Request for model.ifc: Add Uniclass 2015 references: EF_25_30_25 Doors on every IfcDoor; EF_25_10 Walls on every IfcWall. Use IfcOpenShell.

First a look at what the model holds.

```python
import ifcopenshell

model = ifcopenshell.open("model.ifc")
print(model.schema)
print("classifications:", [c.Name for c in model.by_type("IfcClassification")])
for ifc_class in ("IfcDoor", "IfcRoof", "IfcStair", "IfcWall", "IfcWindow"):
    print(ifc_class, len(model.by_type(ifc_class)))
```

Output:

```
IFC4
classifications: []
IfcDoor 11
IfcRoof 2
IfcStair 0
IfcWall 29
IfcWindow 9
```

```python
import ifcopenshell
import ifcopenshell.api.classification

model = ifcopenshell.open("model.ifc")

system = ifcopenshell.api.classification.add_classification(model, classification="Uniclass 2015")

codes = {
    "IfcDoor": ("EF_25_30_25", "Doors"),
    "IfcWall": ("EF_25_10", "Walls"),
}
for ifc_class, (code, name) in codes.items():
    products = model.by_type(ifc_class)
    ifcopenshell.api.classification.add_reference(
        model, products=products, classification=system, identification=code, name=name
    )
    print(code, len(products))

model.write("model-out.ifc")
```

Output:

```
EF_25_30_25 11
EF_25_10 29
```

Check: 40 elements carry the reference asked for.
